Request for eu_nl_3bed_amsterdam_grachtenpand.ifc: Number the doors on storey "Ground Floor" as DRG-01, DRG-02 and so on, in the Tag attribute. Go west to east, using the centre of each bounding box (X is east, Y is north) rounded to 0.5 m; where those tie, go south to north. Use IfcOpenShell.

First a look at what the model holds.

```python
import ifcopenshell
import ifcopenshell.util.element
import ifcopenshell.util.placement

model = ifcopenshell.open("eu_nl_3bed_amsterdam_grachtenpand.ifc")
print(model.schema)
storey = next(s for s in model.by_type("IfcBuildingStorey") if s.Name == "Ground Floor")
doors = [e for e in ifcopenshell.util.element.get_decomposition(storey) if e.is_a("IfcDoor")]
for e in sorted(doors, key=lambda e: e.id()):
    origin = ifcopenshell.util.placement.get_local_placement(e.ObjectPlacement)[:3, 3]
    print(e.id(), e.Tag, e.Name, origin.round(2) + 0.0, sep=" | ")
```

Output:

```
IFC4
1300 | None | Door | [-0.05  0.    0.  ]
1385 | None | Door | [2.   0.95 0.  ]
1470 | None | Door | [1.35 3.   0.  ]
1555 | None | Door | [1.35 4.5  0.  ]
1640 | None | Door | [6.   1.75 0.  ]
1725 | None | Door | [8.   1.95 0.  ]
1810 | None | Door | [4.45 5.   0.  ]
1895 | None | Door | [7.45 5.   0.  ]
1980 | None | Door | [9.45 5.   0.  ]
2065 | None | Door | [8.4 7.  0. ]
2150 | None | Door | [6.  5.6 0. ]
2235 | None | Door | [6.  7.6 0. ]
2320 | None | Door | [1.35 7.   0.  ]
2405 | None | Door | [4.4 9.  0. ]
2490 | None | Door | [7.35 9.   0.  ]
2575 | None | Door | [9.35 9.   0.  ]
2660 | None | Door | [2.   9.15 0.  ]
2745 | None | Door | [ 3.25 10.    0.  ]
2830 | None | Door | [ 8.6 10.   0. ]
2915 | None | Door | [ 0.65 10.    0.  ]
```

```python
import ifcopenshell
import ifcopenshell.geom
import ifcopenshell.util.element
import ifcopenshell.util.shape

model = ifcopenshell.open("eu_nl_3bed_amsterdam_grachtenpand.ifc")
settings = ifcopenshell.geom.settings()
settings.set("use-world-coords", True)


def centre(element):
    shape = ifcopenshell.geom.create_shape(settings, element)
    return ifcopenshell.util.shape.get_bbox_centroid(shape.geometry)


storey = next(s for s in model.by_type("IfcBuildingStorey") if s.Name == "Ground Floor")
doors = [e for e in ifcopenshell.util.element.get_decomposition(storey) if e.is_a("IfcDoor")]

# Insertion points can sit at a corner or the storey origin, so sort by the geometry (in metres).
centres = {e: centre(e) for e in doors}
doors.sort(key=lambda e: (round(centres[e][0] / 0.5), centres[e][1]))

for i, e in enumerate(doors, start=1):
    number = f"DRG-{i:02d}"
    e.Tag = number
    print(e.id(), number)

model.write("eu_nl_3bed_amsterdam_grachtenpand_updated.ifc")
```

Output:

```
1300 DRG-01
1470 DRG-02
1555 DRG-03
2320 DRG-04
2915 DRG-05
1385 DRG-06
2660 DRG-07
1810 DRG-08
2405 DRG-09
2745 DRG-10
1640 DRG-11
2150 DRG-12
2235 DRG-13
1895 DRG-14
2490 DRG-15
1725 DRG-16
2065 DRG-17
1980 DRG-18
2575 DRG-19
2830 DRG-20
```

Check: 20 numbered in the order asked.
